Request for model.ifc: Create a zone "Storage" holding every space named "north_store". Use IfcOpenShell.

First a look at what the model holds.

```python
import ifcopenshell

model = ifcopenshell.open("model.ifc")
print(model.schema)
seen = {}
for space in model.by_type("IfcSpace"):
    seen[space.Name] = seen.get(space.Name, 0) + 1
for name, count in sorted(seen.items(), key=str):
    print(count, "x", name)
print("zones:", [z.Name for z in model.by_type("IfcZone")][:20])
```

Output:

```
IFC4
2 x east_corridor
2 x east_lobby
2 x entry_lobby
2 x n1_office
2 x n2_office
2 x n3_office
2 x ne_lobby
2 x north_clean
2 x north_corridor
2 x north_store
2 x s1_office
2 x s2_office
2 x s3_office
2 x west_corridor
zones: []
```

```python
import ifcopenshell
import ifcopenshell.api.group
import ifcopenshell.api.root

model = ifcopenshell.open("model.ifc")

names = {"north_store"}
spaces = [s for s in model.by_type("IfcSpace") if s.Name in names]

zone = ifcopenshell.api.root.create_entity(model, ifc_class="IfcZone", name="Storage")
ifcopenshell.api.group.assign_group(model, products=spaces, group=zone)
print(len(spaces), "spaces in", zone.Name)

model.write("model_rev.ifc")
```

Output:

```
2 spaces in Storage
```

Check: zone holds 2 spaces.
